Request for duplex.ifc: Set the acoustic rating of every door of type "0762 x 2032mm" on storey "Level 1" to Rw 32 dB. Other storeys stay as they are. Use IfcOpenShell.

First a look at what the model holds.

```python
import ifcopenshell
import ifcopenshell.util.element

model = ifcopenshell.open("duplex.ifc")
print(model.schema)
storey = next(s for s in model.by_type("IfcBuildingStorey") if s.Name == "Level 1")
doors = [e for e in ifcopenshell.util.element.get_decomposition(storey) if e.is_a("IfcDoor")]
seen = {}
for e in doors:
    element_type = ifcopenshell.util.element.get_type(e)
    key = (element_type.Name if element_type != e and element_type else None, ifcopenshell.util.element.get_pset(e, "Pset_DoorCommon", "AcousticRating"))
    seen[key] = seen.get(key, 0) + 1
for (name, value), count in sorted(seen.items(), key=str):
    print(count, "x", name, "|", value)
```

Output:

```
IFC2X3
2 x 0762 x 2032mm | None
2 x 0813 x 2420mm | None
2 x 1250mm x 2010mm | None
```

```python
import ifcopenshell
import ifcopenshell.api.pset
import ifcopenshell.util.element

model = ifcopenshell.open("duplex.ifc")

storey = next(s for s in model.by_type("IfcBuildingStorey") if s.Name == "Level 1")
doors = [e for e in ifcopenshell.util.element.get_decomposition(storey) if e.is_a("IfcDoor")]

count = 0
for e in doors:
    element_type = ifcopenshell.util.element.get_type(e)
    if element_type in (None, e) or element_type.Name != "0762 x 2032mm":
        continue
    # add_pset returns the element's existing set when there is one.
    pset = ifcopenshell.api.pset.add_pset(model, product=e, name="Pset_DoorCommon")
    ifcopenshell.api.pset.edit_pset(model, pset=pset, properties={"AcousticRating": "Rw 32 dB"})
    count += 1

print(count, "doors updated")

model.write("duplex_rev.ifc")
```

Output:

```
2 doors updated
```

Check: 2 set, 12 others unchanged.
